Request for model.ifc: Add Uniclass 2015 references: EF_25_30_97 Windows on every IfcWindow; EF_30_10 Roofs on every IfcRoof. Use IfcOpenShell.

First a look at what the model holds.

```python
import ifcopenshell

model = ifcopenshell.open("model.ifc")
print(model.schema)
print("classifications:", [c.Name for c in model.by_type("IfcClassification")])
for ifc_class in ("IfcDoor", "IfcRoof", "IfcStair", "IfcWall", "IfcWindow"):
    print(ifc_class, len(model.by_type(ifc_class)))
```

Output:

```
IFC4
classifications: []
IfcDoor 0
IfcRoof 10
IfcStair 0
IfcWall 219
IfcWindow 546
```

```python
import ifcopenshell
import ifcopenshell.api.classification

model = ifcopenshell.open("model.ifc")

system = ifcopenshell.api.classification.add_classification(model, classification="Uniclass 2015")

codes = {
    "IfcWindow": ("EF_25_30_97", "Windows"),
    "IfcRoof": ("EF_30_10", "Roofs"),
}
for ifc_class, (code, name) in codes.items():
    products = model.by_type(ifc_class)
    ifcopenshell.api.classification.add_reference(
        model, products=products, classification=system, identification=code, name=name
    )
    print(code, len(products))

model.write("model_edited.ifc")
```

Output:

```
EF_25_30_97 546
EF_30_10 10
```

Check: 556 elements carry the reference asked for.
